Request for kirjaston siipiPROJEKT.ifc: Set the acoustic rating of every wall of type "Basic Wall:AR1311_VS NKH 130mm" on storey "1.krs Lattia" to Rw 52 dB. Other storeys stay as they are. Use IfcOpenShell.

First a look at what the model holds.

```python
import ifcopenshell
import ifcopenshell.util.element

model = ifcopenshell.open("kirjaston siipiPROJEKT.ifc")
print(model.schema)
storey = next(s for s in model.by_type("IfcBuildingStorey") if s.Name == "1.krs Lattia")
walls = [e for e in ifcopenshell.util.element.get_decomposition(storey) if e.is_a("IfcWall")]
seen = {}
for e in walls:
    element_type = ifcopenshell.util.element.get_type(e)
    key = (element_type.Name if element_type != e and element_type else None, ifcopenshell.util.element.get_pset(e, "Pset_WallCommon", "AcousticRating"))
    seen[key] = seen.get(key, 0) + 1
for (name, value), count in sorted(seen.items(), key=str):
    print(count, "x", name, "|", value)
```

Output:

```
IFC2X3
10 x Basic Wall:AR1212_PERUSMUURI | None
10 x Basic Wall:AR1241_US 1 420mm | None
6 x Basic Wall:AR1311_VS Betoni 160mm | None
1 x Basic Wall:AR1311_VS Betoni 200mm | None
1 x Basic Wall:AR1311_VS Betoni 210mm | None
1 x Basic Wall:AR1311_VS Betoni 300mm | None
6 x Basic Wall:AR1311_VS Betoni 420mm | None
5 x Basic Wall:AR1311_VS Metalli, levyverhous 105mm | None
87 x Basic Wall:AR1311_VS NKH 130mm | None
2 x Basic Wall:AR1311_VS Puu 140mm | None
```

```python
import ifcopenshell
import ifcopenshell.api.pset
import ifcopenshell.util.element

model = ifcopenshell.open("kirjaston siipiPROJEKT.ifc")

storey = next(s for s in model.by_type("IfcBuildingStorey") if s.Name == "1.krs Lattia")
walls = [e for e in ifcopenshell.util.element.get_decomposition(storey) if e.is_a("IfcWall")]

count = 0
for e in walls:
    element_type = ifcopenshell.util.element.get_type(e)
    if element_type in (None, e) or element_type.Name != "Basic Wall:AR1311_VS NKH 130mm":
        continue
    # add_pset returns the element's existing set when there is one.
    pset = ifcopenshell.api.pset.add_pset(model, product=e, name="Pset_WallCommon")
    ifcopenshell.api.pset.edit_pset(model, pset=pset, properties={"AcousticRating": "Rw 52 dB"})
    count += 1

print(count, "walls updated")

model.write("kirjaston siipiPROJEKT_edited.ifc")
```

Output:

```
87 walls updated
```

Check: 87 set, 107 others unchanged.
